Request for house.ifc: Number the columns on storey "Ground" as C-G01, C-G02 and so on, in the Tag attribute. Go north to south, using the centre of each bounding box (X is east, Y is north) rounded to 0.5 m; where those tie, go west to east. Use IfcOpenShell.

First a look at what the model holds.

```python
import ifcopenshell
import ifcopenshell.util.element
import ifcopenshell.util.placement

model = ifcopenshell.open("house.ifc")
print(model.schema)
storey = next(s for s in model.by_type("IfcBuildingStorey") if s.Name == "Ground")
columns = [e for e in ifcopenshell.util.element.get_decomposition(storey) if e.is_a("IfcColumn")]
for e in sorted(columns, key=lambda e: e.id()):
    origin = ifcopenshell.util.placement.get_local_placement(e.ObjectPlacement)[:3, 3]
    print(e.id(), e.Tag, e.Name, origin.round(2) + 0.0, sep=" | ")
```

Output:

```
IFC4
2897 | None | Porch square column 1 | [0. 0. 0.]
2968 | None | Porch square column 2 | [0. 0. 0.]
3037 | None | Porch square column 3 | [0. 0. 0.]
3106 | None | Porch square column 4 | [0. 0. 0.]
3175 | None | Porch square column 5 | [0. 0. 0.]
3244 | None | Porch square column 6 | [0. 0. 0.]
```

```python
import ifcopenshell
import ifcopenshell.geom
import ifcopenshell.util.element
import ifcopenshell.util.shape

model = ifcopenshell.open("house.ifc")
settings = ifcopenshell.geom.settings()
settings.set("use-world-coords", True)


def centre(element):
    shape = ifcopenshell.geom.create_shape(settings, element)
    return ifcopenshell.util.shape.get_bbox_centroid(shape.geometry)


storey = next(s for s in model.by_type("IfcBuildingStorey") if s.Name == "Ground")
columns = [e for e in ifcopenshell.util.element.get_decomposition(storey) if e.is_a("IfcColumn")]

# Insertion points can sit at a corner or the storey origin, so sort by the geometry (in metres).
centres = {e: centre(e) for e in columns}
columns.sort(key=lambda e: (-round(centres[e][1] / 0.5), centres[e][0]))

for i, e in enumerate(columns, start=1):
    number = f"C-G{i:02d}"
    e.Tag = number
    print(e.id(), number)

model.write("house_updated.ifc")
```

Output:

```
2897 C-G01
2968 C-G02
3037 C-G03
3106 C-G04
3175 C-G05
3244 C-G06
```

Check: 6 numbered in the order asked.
